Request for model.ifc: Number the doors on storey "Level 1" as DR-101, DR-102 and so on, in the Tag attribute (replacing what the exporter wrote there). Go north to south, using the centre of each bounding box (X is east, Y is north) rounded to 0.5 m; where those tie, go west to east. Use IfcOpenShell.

First a look at what the model holds.

```python
import ifcopenshell
import ifcopenshell.util.element
import ifcopenshell.util.placement

model = ifcopenshell.open("model.ifc")
print(model.schema)
storey = next(s for s in model.by_type("IfcBuildingStorey") if s.Name == "Level 1")
doors = [e for e in ifcopenshell.util.element.get_decomposition(storey) if e.is_a("IfcDoor")]
for e in sorted(doors, key=lambda e: e.id()):
    origin = ifcopenshell.util.placement.get_local_placement(e.ObjectPlacement)[:3, 3]
    print(e.id(), e.Tag, e.Name, origin.round(2) + 0.0, sep=" | ")
```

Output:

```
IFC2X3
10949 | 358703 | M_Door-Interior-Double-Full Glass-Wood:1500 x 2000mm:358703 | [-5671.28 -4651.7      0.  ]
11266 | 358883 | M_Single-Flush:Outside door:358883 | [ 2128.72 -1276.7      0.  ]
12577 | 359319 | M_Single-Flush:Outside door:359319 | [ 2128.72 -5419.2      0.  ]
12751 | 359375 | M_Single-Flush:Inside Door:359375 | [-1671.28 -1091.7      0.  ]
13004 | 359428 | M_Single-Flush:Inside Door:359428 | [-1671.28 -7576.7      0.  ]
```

```python
import ifcopenshell
import ifcopenshell.geom
import ifcopenshell.util.element
import ifcopenshell.util.shape

model = ifcopenshell.open("model.ifc")
settings = ifcopenshell.geom.settings()
settings.set("use-world-coords", True)


def centre(element):
    shape = ifcopenshell.geom.create_shape(settings, element)
    return ifcopenshell.util.shape.get_bbox_centroid(shape.geometry)


storey = next(s for s in model.by_type("IfcBuildingStorey") if s.Name == "Level 1")
doors = [e for e in ifcopenshell.util.element.get_decomposition(storey) if e.is_a("IfcDoor")]

# Insertion points can sit at a corner or the storey origin, so sort by the geometry (in metres).
centres = {e: centre(e) for e in doors}
doors.sort(key=lambda e: (-round(centres[e][1] / 0.5), centres[e][0]))

for i, e in enumerate(doors, start=1):
    number = f"DR-1{i:02d}"
    e.Tag = number
    print(e.id(), number)

model.write("model_updated.ifc")
```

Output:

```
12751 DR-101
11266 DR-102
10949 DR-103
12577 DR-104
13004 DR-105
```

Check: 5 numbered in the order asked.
